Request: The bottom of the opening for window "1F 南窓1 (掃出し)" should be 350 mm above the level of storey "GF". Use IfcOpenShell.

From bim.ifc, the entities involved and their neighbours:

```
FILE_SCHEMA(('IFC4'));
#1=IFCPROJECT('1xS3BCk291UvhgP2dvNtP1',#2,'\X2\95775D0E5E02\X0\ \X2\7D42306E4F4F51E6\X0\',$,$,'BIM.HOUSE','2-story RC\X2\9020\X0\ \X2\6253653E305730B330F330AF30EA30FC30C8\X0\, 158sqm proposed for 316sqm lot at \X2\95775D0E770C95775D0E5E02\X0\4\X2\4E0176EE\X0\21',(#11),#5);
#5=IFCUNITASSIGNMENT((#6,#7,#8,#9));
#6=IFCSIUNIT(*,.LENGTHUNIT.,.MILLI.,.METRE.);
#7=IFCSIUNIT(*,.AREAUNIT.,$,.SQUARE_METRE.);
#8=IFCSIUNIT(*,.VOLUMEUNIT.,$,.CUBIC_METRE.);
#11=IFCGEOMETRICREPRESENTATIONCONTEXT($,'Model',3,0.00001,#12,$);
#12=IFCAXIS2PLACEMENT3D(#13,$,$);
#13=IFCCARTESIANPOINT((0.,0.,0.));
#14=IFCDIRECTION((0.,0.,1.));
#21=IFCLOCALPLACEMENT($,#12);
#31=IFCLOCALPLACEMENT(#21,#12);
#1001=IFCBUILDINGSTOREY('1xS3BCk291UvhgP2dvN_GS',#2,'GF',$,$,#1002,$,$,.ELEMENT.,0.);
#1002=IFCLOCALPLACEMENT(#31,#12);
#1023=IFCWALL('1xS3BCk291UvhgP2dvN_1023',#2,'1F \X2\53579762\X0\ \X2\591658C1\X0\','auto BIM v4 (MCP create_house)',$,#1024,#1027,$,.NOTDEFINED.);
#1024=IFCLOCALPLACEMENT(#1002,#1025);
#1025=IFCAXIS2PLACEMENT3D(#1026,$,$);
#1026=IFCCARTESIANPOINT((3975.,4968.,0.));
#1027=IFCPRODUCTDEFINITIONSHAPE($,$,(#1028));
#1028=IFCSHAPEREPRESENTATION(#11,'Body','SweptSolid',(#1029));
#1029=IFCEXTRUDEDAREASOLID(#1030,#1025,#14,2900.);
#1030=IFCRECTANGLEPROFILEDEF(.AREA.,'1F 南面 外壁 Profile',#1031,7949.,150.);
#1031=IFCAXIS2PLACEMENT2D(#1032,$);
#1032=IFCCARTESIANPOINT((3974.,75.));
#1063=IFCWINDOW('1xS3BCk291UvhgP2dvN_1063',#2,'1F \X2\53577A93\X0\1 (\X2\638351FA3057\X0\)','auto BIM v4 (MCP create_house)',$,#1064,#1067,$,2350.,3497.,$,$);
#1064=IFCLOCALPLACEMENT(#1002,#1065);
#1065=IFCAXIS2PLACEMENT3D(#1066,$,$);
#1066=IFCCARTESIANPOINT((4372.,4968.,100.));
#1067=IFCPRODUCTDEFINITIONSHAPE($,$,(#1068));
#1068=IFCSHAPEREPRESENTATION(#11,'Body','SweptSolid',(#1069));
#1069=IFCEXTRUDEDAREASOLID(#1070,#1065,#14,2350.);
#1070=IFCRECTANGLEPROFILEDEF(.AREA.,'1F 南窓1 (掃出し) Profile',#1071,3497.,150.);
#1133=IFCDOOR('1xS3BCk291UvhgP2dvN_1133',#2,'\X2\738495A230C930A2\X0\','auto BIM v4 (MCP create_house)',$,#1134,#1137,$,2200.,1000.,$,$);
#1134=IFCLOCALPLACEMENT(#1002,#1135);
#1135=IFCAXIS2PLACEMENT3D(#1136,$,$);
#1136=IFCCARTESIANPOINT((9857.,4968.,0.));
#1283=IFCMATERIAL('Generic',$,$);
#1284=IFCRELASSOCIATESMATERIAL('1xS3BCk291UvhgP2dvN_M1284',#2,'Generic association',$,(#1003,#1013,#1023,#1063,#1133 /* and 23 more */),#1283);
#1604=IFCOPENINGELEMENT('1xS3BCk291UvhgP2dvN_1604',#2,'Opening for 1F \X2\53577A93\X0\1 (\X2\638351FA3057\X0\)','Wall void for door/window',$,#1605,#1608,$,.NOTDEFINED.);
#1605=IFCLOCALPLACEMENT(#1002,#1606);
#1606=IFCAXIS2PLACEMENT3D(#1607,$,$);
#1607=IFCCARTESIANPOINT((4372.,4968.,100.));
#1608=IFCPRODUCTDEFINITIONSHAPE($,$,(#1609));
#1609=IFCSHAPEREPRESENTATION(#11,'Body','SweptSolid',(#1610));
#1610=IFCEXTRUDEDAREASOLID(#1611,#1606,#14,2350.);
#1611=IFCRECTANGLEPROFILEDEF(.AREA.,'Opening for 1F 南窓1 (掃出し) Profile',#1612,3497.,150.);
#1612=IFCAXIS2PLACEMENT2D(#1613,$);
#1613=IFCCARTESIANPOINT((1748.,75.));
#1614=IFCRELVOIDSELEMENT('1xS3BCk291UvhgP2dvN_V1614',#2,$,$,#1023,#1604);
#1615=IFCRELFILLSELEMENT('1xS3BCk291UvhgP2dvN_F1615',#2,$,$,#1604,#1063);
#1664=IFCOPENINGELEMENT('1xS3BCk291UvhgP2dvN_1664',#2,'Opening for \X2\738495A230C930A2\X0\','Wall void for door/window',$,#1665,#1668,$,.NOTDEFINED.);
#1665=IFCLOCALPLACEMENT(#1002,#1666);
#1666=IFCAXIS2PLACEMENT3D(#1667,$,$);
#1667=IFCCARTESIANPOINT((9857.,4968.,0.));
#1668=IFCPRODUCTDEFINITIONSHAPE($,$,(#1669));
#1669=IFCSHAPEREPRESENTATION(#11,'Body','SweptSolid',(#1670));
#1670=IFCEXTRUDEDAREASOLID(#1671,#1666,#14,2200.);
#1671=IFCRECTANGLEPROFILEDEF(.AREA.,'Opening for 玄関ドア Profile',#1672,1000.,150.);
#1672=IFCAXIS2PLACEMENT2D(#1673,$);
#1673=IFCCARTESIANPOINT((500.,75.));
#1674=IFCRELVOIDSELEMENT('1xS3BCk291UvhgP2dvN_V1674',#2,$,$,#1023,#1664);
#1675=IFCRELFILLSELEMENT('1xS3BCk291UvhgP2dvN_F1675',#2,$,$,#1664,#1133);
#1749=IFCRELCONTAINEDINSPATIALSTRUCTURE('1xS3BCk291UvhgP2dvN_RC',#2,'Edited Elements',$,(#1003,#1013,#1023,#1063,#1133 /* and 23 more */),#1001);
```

```python
import numpy as np
import ifcopenshell
import ifcopenshell.api.geometry
import ifcopenshell.geom
import ifcopenshell.util.element
import ifcopenshell.util.placement
import ifcopenshell.util.shape
import ifcopenshell.util.unit

model = ifcopenshell.open("bim.ifc")
unit_scale = ifcopenshell.util.unit.calculate_unit_scale(model)

window = model.by_guid("1xS3BCk291UvhgP2dvN_1063")
opening = window.FillsVoids[0].RelatingOpeningElement
storey = ifcopenshell.util.element.get_container(window, ifc_class="IfcBuildingStorey")
level = ifcopenshell.util.placement.get_local_placement(storey.ObjectPlacement)[2, 3]

# The opening's origin need not be at the sill, so measure its lowest point.
shape = ifcopenshell.geom.create_shape(ifcopenshell.geom.settings(), opening)
bottom = ifcopenshell.util.shape.get_shape_bottom_elevation(shape, shape.geometry) / unit_scale
dz = level + 0.35 / unit_scale - bottom

shift = np.array([0.0, 0.0, dz])
# The window is not placed relative to its opening, so move both.
for product in (opening, window):
    matrix = ifcopenshell.util.placement.get_local_placement(product.ObjectPlacement)
    matrix[:3, 3] += shift
    ifcopenshell.api.geometry.edit_object_placement(model, product=product, matrix=matrix, is_si=False)

print(f"moved by {dz * unit_scale:+.3f} m")

model.write("bim_rev.ifc")
```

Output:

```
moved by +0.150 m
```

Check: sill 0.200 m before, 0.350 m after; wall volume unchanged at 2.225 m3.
